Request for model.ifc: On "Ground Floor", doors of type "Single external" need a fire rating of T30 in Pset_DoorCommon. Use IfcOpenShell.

First a look at what the model holds.

```python
import ifcopenshell
import ifcopenshell.util.element

model = ifcopenshell.open("model.ifc")
print(model.schema)
storey = next(s for s in model.by_type("IfcBuildingStorey") if s.Name == "Ground Floor")
doors = [e for e in ifcopenshell.util.element.get_decomposition(storey) if e.is_a("IfcDoor")]
seen = {}
for e in doors:
    element_type = ifcopenshell.util.element.get_type(e)
    key = (element_type.Name if element_type != e and element_type else None, ifcopenshell.util.element.get_pset(e, "Pset_DoorCommon", "FireRating"))
    seen[key] = seen.get(key, 0) + 1
for (name, value), count in sorted(seen.items(), key=str):
    print(count, "x", name, "|", value)
```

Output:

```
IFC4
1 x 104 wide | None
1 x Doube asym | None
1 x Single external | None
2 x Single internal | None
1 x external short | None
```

```python
import ifcopenshell
import ifcopenshell.api.pset
import ifcopenshell.util.element

model = ifcopenshell.open("model.ifc")

storey = next(s for s in model.by_type("IfcBuildingStorey") if s.Name == "Ground Floor")
doors = [e for e in ifcopenshell.util.element.get_decomposition(storey) if e.is_a("IfcDoor")]

count = 0
for e in doors:
    element_type = ifcopenshell.util.element.get_type(e)
    if element_type in (None, e) or element_type.Name != "Single external":
        continue
    # add_pset returns the element's existing set when there is one.
    pset = ifcopenshell.api.pset.add_pset(model, product=e, name="Pset_DoorCommon")
    ifcopenshell.api.pset.edit_pset(model, pset=pset, properties={"FireRating": "T30"})
    count += 1

print(count, "doors updated")

model.write("model_rev.ifc")
```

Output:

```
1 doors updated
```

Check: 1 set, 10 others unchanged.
